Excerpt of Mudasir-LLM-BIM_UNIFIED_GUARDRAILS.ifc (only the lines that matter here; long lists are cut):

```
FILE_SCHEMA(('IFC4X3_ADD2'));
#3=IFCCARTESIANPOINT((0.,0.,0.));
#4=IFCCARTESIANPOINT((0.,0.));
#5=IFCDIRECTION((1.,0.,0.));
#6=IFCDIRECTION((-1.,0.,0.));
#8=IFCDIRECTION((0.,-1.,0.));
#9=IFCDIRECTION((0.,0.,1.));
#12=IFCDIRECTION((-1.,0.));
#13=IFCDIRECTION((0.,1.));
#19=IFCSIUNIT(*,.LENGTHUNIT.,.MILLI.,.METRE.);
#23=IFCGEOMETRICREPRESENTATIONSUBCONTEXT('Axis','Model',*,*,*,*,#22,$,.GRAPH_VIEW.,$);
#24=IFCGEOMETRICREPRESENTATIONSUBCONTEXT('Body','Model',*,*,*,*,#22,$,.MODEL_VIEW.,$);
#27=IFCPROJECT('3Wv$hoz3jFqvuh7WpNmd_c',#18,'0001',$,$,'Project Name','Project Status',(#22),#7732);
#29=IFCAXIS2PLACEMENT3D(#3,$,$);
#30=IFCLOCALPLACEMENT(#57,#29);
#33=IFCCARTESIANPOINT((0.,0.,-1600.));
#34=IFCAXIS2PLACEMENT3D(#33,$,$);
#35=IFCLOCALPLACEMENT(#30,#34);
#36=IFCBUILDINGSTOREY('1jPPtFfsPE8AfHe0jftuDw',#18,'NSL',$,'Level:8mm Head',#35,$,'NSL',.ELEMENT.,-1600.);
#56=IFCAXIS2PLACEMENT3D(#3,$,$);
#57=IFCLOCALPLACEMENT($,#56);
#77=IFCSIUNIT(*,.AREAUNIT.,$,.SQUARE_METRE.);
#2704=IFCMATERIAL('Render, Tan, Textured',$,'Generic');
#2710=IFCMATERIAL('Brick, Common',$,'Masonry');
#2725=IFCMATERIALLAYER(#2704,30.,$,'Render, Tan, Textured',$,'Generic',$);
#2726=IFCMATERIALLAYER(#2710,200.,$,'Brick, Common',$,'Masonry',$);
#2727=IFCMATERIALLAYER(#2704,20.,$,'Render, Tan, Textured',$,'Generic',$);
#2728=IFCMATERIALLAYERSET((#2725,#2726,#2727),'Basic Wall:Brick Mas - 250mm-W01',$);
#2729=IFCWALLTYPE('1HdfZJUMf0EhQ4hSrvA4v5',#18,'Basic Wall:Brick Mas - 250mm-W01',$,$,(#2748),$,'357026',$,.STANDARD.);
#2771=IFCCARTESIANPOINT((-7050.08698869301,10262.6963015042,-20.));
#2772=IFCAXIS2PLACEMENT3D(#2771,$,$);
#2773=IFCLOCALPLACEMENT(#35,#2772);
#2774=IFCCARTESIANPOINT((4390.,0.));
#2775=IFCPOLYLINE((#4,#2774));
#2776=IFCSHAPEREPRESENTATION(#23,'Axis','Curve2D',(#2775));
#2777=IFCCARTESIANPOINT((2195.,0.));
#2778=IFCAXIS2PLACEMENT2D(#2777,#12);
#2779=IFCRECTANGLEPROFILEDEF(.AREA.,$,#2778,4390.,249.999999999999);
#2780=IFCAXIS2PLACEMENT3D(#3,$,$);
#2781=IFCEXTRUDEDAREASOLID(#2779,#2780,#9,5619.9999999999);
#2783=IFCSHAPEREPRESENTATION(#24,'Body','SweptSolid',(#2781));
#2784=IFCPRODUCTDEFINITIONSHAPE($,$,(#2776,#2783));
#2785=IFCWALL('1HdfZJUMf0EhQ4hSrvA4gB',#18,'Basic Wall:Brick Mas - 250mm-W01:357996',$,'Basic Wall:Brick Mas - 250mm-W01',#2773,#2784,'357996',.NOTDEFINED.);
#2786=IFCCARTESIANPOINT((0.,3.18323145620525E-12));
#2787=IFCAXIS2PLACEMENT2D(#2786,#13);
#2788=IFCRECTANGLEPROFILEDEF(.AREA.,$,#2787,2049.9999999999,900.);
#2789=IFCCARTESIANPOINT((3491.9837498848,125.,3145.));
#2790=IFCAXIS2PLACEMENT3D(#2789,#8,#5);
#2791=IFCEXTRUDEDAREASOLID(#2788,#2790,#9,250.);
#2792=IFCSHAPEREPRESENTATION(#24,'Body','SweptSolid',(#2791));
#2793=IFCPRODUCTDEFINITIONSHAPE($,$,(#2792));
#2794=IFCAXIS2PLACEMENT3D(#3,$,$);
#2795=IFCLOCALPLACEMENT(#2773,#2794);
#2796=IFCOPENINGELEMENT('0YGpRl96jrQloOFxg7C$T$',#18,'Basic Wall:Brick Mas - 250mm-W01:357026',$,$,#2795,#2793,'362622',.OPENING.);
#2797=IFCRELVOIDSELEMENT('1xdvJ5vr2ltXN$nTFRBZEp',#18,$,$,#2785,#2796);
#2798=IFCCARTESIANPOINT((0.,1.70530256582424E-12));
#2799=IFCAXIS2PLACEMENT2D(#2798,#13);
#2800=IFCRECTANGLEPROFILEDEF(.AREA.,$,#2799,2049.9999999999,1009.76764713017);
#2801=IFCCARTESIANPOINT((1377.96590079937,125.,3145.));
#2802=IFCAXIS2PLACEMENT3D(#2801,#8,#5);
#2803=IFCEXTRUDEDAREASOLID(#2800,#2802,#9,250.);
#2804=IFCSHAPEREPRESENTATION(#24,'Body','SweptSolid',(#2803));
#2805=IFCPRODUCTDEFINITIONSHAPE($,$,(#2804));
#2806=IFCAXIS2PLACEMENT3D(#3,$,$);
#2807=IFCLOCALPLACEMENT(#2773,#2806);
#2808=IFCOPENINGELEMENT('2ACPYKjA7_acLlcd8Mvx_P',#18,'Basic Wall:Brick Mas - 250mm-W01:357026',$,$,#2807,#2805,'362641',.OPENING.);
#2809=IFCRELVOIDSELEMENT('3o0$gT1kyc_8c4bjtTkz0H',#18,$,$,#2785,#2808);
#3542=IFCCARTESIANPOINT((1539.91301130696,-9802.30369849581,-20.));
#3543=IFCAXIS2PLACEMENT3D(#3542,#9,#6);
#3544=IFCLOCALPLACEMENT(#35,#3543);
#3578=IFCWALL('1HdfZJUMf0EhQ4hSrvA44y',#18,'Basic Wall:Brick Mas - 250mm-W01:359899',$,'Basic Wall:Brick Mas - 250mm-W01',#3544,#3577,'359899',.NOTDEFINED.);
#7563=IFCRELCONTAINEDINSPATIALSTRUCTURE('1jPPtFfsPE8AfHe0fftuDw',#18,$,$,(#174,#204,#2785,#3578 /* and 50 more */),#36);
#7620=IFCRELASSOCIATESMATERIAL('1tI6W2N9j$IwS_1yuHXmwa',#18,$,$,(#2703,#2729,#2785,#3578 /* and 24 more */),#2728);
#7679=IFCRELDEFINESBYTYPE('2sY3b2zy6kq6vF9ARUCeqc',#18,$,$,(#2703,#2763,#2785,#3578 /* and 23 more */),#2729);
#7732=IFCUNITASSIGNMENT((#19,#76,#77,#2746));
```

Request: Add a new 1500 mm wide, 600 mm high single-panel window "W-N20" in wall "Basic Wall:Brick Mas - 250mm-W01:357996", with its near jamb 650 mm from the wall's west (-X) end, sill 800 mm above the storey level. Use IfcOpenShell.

```python
import numpy as np
import ifcopenshell
import ifcopenshell.api.feature
import ifcopenshell.api.geometry
import ifcopenshell.api.root
import ifcopenshell.api.spatial
import ifcopenshell.geom
import ifcopenshell.util.element
import ifcopenshell.util.placement
import ifcopenshell.util.representation
import ifcopenshell.util.shape
import ifcopenshell.util.unit

model = ifcopenshell.open("Mudasir-LLM-BIM_UNIFIED_GUARDRAILS.ifc")
unit_scale = ifcopenshell.util.unit.calculate_unit_scale(model)
settings = ifcopenshell.geom.settings()


def volume(element):
    """Net volume in cubic metres, openings subtracted."""
    shape = ifcopenshell.geom.create_shape(settings, element)
    return ifcopenshell.util.shape.get_volume(shape.geometry)


wall = model.by_guid("1HdfZJUMf0EhQ4hSrvA4gB")
storey = ifcopenshell.util.element.get_container(wall, ifc_class="IfcBuildingStorey")
context = ifcopenshell.util.representation.get_context(model, "Model", "Body", "MODEL_VIEW")
before = volume(wall)

width, height, from_end, sill = 1.5, 0.6, 0.65, 0.8  # metres

# The wall runs along its own X axis, and the end named is its -X end.
wall_shape = ifcopenshell.geom.create_shape(settings, wall)
x, y, z = ifcopenshell.util.shape.get_vertices(wall_shape.geometry).T
start = x.min() + from_end
face, thickness = float(y.min()), float(y.max() - y.min())
wall_matrix = ifcopenshell.util.placement.get_local_placement(wall.ObjectPlacement)
level = ifcopenshell.util.placement.get_local_placement(storey.ObjectPlacement)[2, 3]


def in_wall(x, y):
    """Placement at x, y metres in the wall's axes, at sill height."""
    matrix = wall_matrix.copy()
    matrix[:, 3] = wall_matrix @ np.array([x / unit_scale, y / unit_scale, 0.0, 1.0])
    matrix[2, 3] = level + sill / unit_scale
    return matrix


# Opening: a box that overshoots both wall faces by 50 mm.
opening = ifcopenshell.api.root.create_entity(model, ifc_class="IfcOpeningElement", predefined_type="OPENING")
box = ifcopenshell.api.geometry.add_wall_representation(
    model, context=context, length=width, height=height, thickness=thickness + 0.1
)
ifcopenshell.api.geometry.assign_representation(model, product=opening, representation=box)
ifcopenshell.api.geometry.edit_object_placement(model, product=opening, matrix=in_wall(start, face - 0.05), is_si=False)
ifcopenshell.api.feature.add_feature(model, feature=opening, element=wall)

window = ifcopenshell.api.root.create_entity(model, ifc_class="IfcWindow", name="W-N20", predefined_type="WINDOW")
window.OverallWidth, window.OverallHeight = width / unit_scale, height / unit_scale
window.PartitioningType = "SINGLE_PANEL"
body = ifcopenshell.api.geometry.add_window_representation(
    model,
    context=context,
    overall_width=window.OverallWidth,
    overall_height=window.OverallHeight,
    partition_type="SINGLE_PANEL",
)
ifcopenshell.api.geometry.assign_representation(model, product=window, representation=body)
ifcopenshell.api.spatial.assign_container(model, products=[window], relating_structure=storey)
ifcopenshell.api.feature.add_filling(model, opening=opening, element=window)

# Centre the window in the wall's thickness.
ifcopenshell.api.geometry.edit_object_placement(model, product=window, matrix=in_wall(start, face), is_si=False)
window_shape = ifcopenshell.geom.create_shape(settings, window)
depth = ifcopenshell.util.shape.get_vertices(window_shape.geometry)[:, 1]
offset = face + thickness / 2 - (depth.min() + depth.max()) / 2
ifcopenshell.api.geometry.edit_object_placement(model, product=window, matrix=in_wall(start, offset), is_si=False)

after = volume(wall)

print(f"wall volume {before:.3f} -> {after:.3f} m3")

model.write("Mudasir-LLM-BIM_UNIFIED_GUARDRAILS-out.ifc")
```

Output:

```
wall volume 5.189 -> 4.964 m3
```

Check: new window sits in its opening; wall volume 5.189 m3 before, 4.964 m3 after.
